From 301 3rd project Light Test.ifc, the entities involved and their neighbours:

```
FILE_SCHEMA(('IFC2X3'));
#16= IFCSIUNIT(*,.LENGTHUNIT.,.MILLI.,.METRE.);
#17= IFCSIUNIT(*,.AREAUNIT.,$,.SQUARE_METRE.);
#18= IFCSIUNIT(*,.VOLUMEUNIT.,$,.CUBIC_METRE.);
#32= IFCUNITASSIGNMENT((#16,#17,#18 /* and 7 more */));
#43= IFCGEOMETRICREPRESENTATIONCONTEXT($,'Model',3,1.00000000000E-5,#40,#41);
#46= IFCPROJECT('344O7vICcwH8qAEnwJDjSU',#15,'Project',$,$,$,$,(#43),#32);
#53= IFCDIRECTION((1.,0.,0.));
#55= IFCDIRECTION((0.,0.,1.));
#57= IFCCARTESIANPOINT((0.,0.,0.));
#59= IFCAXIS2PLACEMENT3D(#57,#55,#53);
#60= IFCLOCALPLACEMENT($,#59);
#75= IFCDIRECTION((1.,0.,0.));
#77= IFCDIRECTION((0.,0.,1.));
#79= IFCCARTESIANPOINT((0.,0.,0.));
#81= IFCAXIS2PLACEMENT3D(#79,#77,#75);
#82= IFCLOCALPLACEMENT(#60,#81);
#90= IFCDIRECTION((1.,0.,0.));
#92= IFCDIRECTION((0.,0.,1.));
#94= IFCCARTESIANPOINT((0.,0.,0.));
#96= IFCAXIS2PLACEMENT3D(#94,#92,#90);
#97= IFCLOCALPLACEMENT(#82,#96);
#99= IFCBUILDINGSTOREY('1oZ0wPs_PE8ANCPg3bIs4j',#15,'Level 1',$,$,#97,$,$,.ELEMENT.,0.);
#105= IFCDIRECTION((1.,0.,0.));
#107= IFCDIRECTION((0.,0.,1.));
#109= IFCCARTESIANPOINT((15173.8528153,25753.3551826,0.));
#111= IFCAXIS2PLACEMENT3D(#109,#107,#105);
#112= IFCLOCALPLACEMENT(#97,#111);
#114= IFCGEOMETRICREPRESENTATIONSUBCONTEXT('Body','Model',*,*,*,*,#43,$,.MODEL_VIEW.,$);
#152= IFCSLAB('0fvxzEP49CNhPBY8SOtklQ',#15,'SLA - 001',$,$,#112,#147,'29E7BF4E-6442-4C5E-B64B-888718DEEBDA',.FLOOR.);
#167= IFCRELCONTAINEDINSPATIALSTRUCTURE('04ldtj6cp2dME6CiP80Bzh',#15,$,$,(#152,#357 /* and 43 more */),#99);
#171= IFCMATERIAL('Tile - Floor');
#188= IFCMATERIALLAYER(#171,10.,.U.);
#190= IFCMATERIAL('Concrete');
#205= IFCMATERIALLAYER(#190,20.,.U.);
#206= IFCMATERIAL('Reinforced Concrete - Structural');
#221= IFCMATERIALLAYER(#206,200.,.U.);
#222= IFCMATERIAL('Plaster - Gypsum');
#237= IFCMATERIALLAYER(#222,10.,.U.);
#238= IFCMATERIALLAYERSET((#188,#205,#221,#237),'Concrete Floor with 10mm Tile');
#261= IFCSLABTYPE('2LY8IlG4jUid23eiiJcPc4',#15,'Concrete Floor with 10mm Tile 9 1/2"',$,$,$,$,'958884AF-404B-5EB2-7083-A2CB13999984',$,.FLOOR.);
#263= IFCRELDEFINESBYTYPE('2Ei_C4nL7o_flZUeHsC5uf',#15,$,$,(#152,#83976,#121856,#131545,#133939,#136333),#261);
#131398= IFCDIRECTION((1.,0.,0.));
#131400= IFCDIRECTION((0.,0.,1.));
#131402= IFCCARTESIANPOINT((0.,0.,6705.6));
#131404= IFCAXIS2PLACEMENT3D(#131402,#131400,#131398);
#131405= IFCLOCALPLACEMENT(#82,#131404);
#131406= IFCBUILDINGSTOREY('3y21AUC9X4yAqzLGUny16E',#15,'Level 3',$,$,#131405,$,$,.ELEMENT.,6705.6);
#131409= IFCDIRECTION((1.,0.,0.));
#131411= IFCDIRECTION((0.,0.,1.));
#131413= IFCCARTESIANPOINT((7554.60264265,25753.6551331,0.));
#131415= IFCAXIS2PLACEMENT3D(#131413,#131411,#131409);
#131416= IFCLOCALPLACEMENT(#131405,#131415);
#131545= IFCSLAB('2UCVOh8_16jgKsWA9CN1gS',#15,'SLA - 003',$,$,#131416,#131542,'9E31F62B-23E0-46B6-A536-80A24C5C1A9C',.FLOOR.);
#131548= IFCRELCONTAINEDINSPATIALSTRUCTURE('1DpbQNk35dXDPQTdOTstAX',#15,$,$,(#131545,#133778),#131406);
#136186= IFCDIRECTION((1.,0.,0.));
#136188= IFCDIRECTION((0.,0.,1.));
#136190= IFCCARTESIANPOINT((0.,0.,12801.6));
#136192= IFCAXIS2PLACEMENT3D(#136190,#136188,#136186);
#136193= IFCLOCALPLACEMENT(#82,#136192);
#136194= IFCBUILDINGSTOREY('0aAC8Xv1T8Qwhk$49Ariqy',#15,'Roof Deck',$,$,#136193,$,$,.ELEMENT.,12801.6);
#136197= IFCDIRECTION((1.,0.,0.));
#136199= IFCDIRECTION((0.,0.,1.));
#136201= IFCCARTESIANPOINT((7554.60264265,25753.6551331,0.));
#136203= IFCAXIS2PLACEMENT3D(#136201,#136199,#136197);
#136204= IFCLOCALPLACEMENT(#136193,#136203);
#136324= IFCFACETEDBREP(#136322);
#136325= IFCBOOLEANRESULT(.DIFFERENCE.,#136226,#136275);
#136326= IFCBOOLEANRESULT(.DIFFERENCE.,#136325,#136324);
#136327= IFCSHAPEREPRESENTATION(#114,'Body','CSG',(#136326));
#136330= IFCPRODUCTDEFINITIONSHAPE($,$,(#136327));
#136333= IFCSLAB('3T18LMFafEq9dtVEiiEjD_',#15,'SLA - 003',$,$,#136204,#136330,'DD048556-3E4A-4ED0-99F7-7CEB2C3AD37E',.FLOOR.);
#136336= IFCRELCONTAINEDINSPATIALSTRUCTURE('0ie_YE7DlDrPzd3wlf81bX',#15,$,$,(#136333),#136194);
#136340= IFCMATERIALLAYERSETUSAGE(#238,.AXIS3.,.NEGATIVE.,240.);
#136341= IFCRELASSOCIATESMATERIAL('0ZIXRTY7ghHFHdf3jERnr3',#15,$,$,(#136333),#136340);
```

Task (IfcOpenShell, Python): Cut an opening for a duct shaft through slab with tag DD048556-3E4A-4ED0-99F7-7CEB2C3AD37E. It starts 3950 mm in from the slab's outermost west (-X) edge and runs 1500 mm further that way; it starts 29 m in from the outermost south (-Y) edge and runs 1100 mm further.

```python
import numpy as np
import ifcopenshell
import ifcopenshell.api.feature
import ifcopenshell.api.geometry
import ifcopenshell.api.root
import ifcopenshell.geom
import ifcopenshell.util.placement
import ifcopenshell.util.representation
import ifcopenshell.util.shape
import ifcopenshell.util.unit

model = ifcopenshell.open("301 3rd project Light Test.ifc")
unit_scale = ifcopenshell.util.unit.calculate_unit_scale(model)
settings = ifcopenshell.geom.settings()


def volume(element):
    """Net volume in cubic metres, openings subtracted."""
    shape = ifcopenshell.geom.create_shape(settings, element)
    return ifcopenshell.util.shape.get_volume(shape.geometry)


slab = model.by_id(136333)
before = volume(slab)

# Extent in the slab's own axes, in metres. The edges named are its -X and -Y sides.
slab_shape = ifcopenshell.geom.create_shape(settings, slab)
vertices = ifcopenshell.util.shape.get_vertices(slab_shape.geometry)
x_min, y_min, bottom = vertices.min(axis=0)
top = vertices[:, 2].max()

opening = ifcopenshell.api.root.create_entity(model, ifc_class="IfcOpeningElement", name="Duct shaft opening")
context = ifcopenshell.util.representation.get_context(model, "Model", "Body", "MODEL_VIEW")
width, depth = 1.5, 1.1
outline = [(0.0, 0.0), (width, 0.0), (width, depth), (0.0, depth), (0.0, 0.0)]
# Overshoot both faces by 50 mm so the cut is clean.
shape = ifcopenshell.api.geometry.add_slab_representation(
    model, context=context, depth=top - bottom + 0.1, polyline=outline
)
ifcopenshell.api.geometry.assign_representation(model, product=opening, representation=shape)

matrix = ifcopenshell.util.placement.get_local_placement(slab.ObjectPlacement)
matrix[:, 3] = matrix @ np.append(np.array([x_min + 3.95, y_min + 29, bottom - 0.05]) / unit_scale, 1.0)
ifcopenshell.api.geometry.edit_object_placement(model, product=opening, matrix=matrix, is_si=False)
ifcopenshell.api.feature.add_feature(model, feature=opening, element=slab)

after = volume(slab)

print(f"slab volume {before:.3f} -> {after:.3f} m3")

model.write("301 3rd project Light Test_v2.ifc")
```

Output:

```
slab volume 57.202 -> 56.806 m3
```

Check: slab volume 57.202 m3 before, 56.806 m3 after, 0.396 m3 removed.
